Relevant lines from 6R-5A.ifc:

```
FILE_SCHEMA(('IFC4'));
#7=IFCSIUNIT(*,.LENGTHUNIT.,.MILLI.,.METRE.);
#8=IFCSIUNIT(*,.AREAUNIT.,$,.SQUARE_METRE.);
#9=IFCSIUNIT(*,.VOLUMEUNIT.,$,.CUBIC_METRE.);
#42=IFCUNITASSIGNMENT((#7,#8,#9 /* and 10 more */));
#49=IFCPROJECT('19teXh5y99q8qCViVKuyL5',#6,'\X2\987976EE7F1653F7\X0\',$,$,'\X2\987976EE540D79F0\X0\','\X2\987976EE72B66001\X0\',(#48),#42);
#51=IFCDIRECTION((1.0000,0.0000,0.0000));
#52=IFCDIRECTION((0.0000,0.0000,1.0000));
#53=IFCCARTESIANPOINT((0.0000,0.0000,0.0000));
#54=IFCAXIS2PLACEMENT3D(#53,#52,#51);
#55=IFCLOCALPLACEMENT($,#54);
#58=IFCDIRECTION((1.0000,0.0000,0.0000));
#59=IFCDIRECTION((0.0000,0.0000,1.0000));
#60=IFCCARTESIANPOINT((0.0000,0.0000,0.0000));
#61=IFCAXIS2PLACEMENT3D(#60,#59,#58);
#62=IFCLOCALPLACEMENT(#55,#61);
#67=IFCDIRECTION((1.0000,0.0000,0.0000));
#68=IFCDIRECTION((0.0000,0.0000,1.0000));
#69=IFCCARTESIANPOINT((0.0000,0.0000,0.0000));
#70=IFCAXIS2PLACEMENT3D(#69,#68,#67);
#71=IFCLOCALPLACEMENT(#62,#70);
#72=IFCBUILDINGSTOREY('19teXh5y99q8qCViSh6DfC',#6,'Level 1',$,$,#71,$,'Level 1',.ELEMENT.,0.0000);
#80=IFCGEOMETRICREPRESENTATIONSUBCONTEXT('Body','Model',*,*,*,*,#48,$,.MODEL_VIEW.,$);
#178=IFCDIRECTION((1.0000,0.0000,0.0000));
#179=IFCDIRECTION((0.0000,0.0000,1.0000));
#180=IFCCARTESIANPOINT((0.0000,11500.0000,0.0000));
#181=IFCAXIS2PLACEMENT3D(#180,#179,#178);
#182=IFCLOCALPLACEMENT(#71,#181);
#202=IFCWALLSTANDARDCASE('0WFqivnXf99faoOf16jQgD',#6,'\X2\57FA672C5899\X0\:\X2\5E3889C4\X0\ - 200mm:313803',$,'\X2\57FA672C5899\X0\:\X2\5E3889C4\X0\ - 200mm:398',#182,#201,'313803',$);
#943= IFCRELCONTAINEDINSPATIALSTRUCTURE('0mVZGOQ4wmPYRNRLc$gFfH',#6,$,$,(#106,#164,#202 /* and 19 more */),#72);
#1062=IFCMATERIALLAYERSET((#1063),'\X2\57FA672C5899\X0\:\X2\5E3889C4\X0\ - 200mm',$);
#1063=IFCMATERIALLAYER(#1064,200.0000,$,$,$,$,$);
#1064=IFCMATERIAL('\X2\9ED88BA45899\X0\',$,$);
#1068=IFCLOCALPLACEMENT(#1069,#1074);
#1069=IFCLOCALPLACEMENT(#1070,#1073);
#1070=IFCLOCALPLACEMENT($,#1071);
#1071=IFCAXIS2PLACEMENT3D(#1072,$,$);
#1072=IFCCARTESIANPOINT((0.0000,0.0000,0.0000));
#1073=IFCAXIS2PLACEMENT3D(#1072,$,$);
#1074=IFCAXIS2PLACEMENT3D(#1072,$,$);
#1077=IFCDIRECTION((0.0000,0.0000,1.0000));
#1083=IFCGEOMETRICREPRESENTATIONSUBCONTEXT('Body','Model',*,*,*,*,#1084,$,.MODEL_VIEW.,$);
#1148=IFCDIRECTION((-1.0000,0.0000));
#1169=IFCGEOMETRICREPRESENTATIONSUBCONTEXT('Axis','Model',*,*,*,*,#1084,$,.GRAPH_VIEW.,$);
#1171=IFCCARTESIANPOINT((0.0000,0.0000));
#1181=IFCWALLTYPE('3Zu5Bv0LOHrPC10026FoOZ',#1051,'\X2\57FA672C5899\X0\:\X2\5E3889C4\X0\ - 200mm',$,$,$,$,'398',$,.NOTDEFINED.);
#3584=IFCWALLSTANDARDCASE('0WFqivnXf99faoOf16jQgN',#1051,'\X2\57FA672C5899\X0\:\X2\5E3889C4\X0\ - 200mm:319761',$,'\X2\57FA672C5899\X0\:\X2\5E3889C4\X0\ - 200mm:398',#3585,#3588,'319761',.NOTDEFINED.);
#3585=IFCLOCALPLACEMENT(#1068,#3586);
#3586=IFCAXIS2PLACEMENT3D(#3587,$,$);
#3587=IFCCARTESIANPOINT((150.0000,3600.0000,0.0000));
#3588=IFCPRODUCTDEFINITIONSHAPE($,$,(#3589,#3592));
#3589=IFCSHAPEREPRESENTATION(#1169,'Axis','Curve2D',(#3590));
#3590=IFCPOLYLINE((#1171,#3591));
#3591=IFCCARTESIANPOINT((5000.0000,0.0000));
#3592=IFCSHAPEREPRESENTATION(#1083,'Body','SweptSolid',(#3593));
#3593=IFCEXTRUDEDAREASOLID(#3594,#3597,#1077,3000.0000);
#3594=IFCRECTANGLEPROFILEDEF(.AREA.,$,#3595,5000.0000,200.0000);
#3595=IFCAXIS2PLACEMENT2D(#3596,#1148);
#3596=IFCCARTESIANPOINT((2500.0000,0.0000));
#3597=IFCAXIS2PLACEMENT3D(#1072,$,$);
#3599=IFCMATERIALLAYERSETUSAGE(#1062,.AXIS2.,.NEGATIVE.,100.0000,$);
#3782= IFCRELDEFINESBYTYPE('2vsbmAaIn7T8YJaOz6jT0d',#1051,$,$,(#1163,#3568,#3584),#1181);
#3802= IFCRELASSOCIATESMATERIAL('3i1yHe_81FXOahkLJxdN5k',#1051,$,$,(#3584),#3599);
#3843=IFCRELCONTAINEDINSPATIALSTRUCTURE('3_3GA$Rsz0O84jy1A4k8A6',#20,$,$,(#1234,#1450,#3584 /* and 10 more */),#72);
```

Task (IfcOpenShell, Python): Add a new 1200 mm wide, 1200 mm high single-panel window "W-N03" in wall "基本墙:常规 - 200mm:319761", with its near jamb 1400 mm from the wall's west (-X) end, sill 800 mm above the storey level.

```python
import numpy as np
import ifcopenshell
import ifcopenshell.api.feature
import ifcopenshell.api.geometry
import ifcopenshell.api.root
import ifcopenshell.api.spatial
import ifcopenshell.geom
import ifcopenshell.util.element
import ifcopenshell.util.placement
import ifcopenshell.util.representation
import ifcopenshell.util.shape
import ifcopenshell.util.unit

model = ifcopenshell.open("6R-5A.ifc")
unit_scale = ifcopenshell.util.unit.calculate_unit_scale(model)
settings = ifcopenshell.geom.settings()


def volume(element):
    """Net volume in cubic metres, openings subtracted."""
    shape = ifcopenshell.geom.create_shape(settings, element)
    return ifcopenshell.util.shape.get_volume(shape.geometry)


wall = model.by_id(3584)
storey = ifcopenshell.util.element.get_container(wall, ifc_class="IfcBuildingStorey")
context = ifcopenshell.util.representation.get_context(model, "Model", "Body", "MODEL_VIEW")
before = volume(wall)

width, height, from_end, sill = 1.2, 1.2, 1.4, 0.8  # metres

# The wall runs along its own X axis, and the end named is its -X end.
wall_shape = ifcopenshell.geom.create_shape(settings, wall)
x, y, z = ifcopenshell.util.shape.get_vertices(wall_shape.geometry).T
start = x.min() + from_end
face, thickness = float(y.min()), float(y.max() - y.min())
wall_matrix = ifcopenshell.util.placement.get_local_placement(wall.ObjectPlacement)
level = ifcopenshell.util.placement.get_local_placement(storey.ObjectPlacement)[2, 3]


def in_wall(x, y):
    """Placement at x, y metres in the wall's axes, at sill height."""
    matrix = wall_matrix.copy()
    matrix[:, 3] = wall_matrix @ np.array([x / unit_scale, y / unit_scale, 0.0, 1.0])
    matrix[2, 3] = level + sill / unit_scale
    return matrix


# Opening: a box that overshoots both wall faces by 50 mm.
opening = ifcopenshell.api.root.create_entity(model, ifc_class="IfcOpeningElement", predefined_type="OPENING")
box = ifcopenshell.api.geometry.add_wall_representation(
    model, context=context, length=width, height=height, thickness=thickness + 0.1
)
ifcopenshell.api.geometry.assign_representation(model, product=opening, representation=box)
ifcopenshell.api.geometry.edit_object_placement(model, product=opening, matrix=in_wall(start, face - 0.05), is_si=False)
ifcopenshell.api.feature.add_feature(model, feature=opening, element=wall)

window = ifcopenshell.api.root.create_entity(model, ifc_class="IfcWindow", name="W-N03", predefined_type="WINDOW")
window.OverallWidth, window.OverallHeight = width / unit_scale, height / unit_scale
window.PartitioningType = "SINGLE_PANEL"
body = ifcopenshell.api.geometry.add_window_representation(
    model,
    context=context,
    overall_width=window.OverallWidth,
    overall_height=window.OverallHeight,
    partition_type="SINGLE_PANEL",
)
ifcopenshell.api.geometry.assign_representation(model, product=window, representation=body)
ifcopenshell.api.spatial.assign_container(model, products=[window], relating_structure=storey)
ifcopenshell.api.feature.add_filling(model, opening=opening, element=window)

# Centre the window in the wall's thickness.
ifcopenshell.api.geometry.edit_object_placement(model, product=window, matrix=in_wall(start, face), is_si=False)
window_shape = ifcopenshell.geom.create_shape(settings, window)
depth = ifcopenshell.util.shape.get_vertices(window_shape.geometry)[:, 1]
offset = face + thickness / 2 - (depth.min() + depth.max()) / 2
ifcopenshell.api.geometry.edit_object_placement(model, product=window, matrix=in_wall(start, offset), is_si=False)

after = volume(wall)

print(f"wall volume {before:.3f} -> {after:.3f} m3")

model.write("6R-5A_updated.ifc")
```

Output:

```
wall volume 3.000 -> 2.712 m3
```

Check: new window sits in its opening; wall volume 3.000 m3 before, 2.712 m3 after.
